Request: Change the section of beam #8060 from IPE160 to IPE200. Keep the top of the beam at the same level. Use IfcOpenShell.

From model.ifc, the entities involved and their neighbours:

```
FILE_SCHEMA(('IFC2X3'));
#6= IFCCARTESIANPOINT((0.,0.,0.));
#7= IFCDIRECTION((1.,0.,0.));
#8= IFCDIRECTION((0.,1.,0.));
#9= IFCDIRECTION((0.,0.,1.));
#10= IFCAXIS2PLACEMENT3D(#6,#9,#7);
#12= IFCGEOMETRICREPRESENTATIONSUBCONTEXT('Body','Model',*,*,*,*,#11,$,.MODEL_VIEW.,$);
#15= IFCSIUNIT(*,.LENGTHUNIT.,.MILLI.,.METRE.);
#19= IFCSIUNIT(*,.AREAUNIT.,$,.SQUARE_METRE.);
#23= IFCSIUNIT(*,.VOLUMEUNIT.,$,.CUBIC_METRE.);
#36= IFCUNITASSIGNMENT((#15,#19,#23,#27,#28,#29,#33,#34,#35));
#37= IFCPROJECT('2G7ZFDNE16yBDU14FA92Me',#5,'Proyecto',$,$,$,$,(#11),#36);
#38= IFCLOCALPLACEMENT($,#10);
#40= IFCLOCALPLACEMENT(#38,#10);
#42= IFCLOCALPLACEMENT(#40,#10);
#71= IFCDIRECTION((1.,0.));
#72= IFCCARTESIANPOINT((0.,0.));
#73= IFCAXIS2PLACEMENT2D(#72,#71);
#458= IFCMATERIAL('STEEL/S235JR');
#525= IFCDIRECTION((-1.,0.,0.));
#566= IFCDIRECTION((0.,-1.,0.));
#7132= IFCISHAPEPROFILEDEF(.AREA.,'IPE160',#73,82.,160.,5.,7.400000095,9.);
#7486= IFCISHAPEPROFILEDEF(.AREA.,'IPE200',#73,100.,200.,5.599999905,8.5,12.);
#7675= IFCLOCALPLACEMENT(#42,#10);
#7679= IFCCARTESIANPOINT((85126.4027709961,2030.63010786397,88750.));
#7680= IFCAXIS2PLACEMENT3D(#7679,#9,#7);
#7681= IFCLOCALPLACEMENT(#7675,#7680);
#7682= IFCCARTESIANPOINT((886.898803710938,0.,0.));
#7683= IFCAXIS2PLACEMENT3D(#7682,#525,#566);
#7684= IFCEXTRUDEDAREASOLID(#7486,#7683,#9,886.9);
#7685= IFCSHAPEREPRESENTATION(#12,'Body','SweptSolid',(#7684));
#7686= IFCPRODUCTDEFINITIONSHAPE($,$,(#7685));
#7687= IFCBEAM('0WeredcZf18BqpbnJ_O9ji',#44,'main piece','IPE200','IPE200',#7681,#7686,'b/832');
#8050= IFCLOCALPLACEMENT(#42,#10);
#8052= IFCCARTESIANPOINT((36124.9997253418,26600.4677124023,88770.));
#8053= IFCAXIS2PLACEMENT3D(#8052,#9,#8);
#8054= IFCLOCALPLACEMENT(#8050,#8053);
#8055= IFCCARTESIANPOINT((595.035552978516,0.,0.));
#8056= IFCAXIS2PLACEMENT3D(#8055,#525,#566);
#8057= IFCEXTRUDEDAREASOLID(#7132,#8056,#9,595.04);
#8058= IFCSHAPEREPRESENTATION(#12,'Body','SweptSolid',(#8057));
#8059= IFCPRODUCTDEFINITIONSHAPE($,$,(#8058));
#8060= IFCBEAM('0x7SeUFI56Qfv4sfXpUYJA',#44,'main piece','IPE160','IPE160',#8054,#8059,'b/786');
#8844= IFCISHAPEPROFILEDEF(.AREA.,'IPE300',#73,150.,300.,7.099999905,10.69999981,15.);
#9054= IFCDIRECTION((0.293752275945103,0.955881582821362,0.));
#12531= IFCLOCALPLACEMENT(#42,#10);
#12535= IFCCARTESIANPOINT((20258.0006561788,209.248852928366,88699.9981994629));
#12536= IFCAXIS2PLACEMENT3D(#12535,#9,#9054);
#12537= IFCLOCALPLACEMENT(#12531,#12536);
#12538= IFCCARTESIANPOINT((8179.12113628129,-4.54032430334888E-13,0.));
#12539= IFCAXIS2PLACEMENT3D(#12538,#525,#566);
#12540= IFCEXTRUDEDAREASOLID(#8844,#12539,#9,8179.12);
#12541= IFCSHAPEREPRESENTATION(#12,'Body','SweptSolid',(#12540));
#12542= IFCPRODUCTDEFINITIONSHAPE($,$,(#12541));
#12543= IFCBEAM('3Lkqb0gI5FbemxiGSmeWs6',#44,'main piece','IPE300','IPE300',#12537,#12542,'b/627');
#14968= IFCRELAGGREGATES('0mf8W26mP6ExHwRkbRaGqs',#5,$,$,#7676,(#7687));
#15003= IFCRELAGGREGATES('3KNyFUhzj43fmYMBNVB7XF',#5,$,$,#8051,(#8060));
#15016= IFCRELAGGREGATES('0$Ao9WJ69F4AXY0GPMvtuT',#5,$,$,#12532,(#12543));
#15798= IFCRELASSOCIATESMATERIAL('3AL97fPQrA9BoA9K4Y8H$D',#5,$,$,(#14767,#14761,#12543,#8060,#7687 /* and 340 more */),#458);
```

```python
import ifcopenshell
import ifcopenshell.util.element
import ifcopenshell.util.representation

model = ifcopenshell.open("model.ifc")

member = model.by_guid("0x7SeUFI56Qfv4sfXpUYJA")
source = next(p for p in model.by_type("IfcIShapeProfileDef") if p.ProfileName == "IPE200")

body = ifcopenshell.util.representation.get_representation(member, "Model", "Body")
solid = body.Items[0]
old_profile = solid.SweptArea

# Copy the section's sizes but keep this member's own profile position.
profile = ifcopenshell.util.element.copy(model, source)
# Profiles are centred, so shift by half the change in depth to hold the top.
shift = (old_profile.OverallDepth - profile.OverallDepth) / 2
x, y = old_profile.Position.Location.Coordinates
up = (0.0, 1.0)  # upwards, in the solid's own plane
location = model.createIfcCartesianPoint((x + up[0] * shift, y + up[1] * shift))
profile.Position = model.createIfcAxis2Placement2D(location, old_profile.Position.RefDirection)
solid.SweptArea = profile
if not model.get_total_inverses(old_profile):
    ifcopenshell.util.element.remove_deep2(model, old_profile)
member.Description = member.Description.replace("IPE160", "IPE200")
member.ObjectType = member.ObjectType.replace("IPE160", "IPE200")

print(solid.SweptArea)

model.write("model-out.ifc")
```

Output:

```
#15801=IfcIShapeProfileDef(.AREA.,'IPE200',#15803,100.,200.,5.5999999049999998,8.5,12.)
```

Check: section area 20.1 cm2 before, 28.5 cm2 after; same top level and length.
